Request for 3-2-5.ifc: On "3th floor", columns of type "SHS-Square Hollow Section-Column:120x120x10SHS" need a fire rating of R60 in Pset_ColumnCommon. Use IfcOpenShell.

First a look at what the model holds.

```python
import ifcopenshell
import ifcopenshell.util.element

model = ifcopenshell.open("3-2-5.ifc")
print(model.schema)
storey = next(s for s in model.by_type("IfcBuildingStorey") if s.Name == "3th floor")
columns = [e for e in ifcopenshell.util.element.get_decomposition(storey) if e.is_a("IfcColumn")]
seen = {}
for e in columns:
    element_type = ifcopenshell.util.element.get_type(e)
    key = (element_type.Name if element_type != e and element_type else None, ifcopenshell.util.element.get_pset(e, "Pset_ColumnCommon", "FireRating"))
    seen[key] = seen.get(key, 0) + 1
for (name, value), count in sorted(seen.items(), key=str):
    print(count, "x", name, "|", value)
```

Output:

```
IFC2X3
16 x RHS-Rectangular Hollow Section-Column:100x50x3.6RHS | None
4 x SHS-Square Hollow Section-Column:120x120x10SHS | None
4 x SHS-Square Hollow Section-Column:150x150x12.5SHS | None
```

```python
import ifcopenshell
import ifcopenshell.api.pset
import ifcopenshell.util.element

model = ifcopenshell.open("3-2-5.ifc")

storey = next(s for s in model.by_type("IfcBuildingStorey") if s.Name == "3th floor")
columns = [e for e in ifcopenshell.util.element.get_decomposition(storey) if e.is_a("IfcColumn")]

count = 0
for e in columns:
    element_type = ifcopenshell.util.element.get_type(e)
    if element_type in (None, e) or element_type.Name != "SHS-Square Hollow Section-Column:120x120x10SHS":
        continue
    # add_pset returns the element's existing set when there is one.
    pset = ifcopenshell.api.pset.add_pset(model, product=e, name="Pset_ColumnCommon")
    ifcopenshell.api.pset.edit_pset(model, pset=pset, properties={"FireRating": "R60"})
    count += 1

print(count, "columns updated")

model.write("3-2-5_rev.ifc")
```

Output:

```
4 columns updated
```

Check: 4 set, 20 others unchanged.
